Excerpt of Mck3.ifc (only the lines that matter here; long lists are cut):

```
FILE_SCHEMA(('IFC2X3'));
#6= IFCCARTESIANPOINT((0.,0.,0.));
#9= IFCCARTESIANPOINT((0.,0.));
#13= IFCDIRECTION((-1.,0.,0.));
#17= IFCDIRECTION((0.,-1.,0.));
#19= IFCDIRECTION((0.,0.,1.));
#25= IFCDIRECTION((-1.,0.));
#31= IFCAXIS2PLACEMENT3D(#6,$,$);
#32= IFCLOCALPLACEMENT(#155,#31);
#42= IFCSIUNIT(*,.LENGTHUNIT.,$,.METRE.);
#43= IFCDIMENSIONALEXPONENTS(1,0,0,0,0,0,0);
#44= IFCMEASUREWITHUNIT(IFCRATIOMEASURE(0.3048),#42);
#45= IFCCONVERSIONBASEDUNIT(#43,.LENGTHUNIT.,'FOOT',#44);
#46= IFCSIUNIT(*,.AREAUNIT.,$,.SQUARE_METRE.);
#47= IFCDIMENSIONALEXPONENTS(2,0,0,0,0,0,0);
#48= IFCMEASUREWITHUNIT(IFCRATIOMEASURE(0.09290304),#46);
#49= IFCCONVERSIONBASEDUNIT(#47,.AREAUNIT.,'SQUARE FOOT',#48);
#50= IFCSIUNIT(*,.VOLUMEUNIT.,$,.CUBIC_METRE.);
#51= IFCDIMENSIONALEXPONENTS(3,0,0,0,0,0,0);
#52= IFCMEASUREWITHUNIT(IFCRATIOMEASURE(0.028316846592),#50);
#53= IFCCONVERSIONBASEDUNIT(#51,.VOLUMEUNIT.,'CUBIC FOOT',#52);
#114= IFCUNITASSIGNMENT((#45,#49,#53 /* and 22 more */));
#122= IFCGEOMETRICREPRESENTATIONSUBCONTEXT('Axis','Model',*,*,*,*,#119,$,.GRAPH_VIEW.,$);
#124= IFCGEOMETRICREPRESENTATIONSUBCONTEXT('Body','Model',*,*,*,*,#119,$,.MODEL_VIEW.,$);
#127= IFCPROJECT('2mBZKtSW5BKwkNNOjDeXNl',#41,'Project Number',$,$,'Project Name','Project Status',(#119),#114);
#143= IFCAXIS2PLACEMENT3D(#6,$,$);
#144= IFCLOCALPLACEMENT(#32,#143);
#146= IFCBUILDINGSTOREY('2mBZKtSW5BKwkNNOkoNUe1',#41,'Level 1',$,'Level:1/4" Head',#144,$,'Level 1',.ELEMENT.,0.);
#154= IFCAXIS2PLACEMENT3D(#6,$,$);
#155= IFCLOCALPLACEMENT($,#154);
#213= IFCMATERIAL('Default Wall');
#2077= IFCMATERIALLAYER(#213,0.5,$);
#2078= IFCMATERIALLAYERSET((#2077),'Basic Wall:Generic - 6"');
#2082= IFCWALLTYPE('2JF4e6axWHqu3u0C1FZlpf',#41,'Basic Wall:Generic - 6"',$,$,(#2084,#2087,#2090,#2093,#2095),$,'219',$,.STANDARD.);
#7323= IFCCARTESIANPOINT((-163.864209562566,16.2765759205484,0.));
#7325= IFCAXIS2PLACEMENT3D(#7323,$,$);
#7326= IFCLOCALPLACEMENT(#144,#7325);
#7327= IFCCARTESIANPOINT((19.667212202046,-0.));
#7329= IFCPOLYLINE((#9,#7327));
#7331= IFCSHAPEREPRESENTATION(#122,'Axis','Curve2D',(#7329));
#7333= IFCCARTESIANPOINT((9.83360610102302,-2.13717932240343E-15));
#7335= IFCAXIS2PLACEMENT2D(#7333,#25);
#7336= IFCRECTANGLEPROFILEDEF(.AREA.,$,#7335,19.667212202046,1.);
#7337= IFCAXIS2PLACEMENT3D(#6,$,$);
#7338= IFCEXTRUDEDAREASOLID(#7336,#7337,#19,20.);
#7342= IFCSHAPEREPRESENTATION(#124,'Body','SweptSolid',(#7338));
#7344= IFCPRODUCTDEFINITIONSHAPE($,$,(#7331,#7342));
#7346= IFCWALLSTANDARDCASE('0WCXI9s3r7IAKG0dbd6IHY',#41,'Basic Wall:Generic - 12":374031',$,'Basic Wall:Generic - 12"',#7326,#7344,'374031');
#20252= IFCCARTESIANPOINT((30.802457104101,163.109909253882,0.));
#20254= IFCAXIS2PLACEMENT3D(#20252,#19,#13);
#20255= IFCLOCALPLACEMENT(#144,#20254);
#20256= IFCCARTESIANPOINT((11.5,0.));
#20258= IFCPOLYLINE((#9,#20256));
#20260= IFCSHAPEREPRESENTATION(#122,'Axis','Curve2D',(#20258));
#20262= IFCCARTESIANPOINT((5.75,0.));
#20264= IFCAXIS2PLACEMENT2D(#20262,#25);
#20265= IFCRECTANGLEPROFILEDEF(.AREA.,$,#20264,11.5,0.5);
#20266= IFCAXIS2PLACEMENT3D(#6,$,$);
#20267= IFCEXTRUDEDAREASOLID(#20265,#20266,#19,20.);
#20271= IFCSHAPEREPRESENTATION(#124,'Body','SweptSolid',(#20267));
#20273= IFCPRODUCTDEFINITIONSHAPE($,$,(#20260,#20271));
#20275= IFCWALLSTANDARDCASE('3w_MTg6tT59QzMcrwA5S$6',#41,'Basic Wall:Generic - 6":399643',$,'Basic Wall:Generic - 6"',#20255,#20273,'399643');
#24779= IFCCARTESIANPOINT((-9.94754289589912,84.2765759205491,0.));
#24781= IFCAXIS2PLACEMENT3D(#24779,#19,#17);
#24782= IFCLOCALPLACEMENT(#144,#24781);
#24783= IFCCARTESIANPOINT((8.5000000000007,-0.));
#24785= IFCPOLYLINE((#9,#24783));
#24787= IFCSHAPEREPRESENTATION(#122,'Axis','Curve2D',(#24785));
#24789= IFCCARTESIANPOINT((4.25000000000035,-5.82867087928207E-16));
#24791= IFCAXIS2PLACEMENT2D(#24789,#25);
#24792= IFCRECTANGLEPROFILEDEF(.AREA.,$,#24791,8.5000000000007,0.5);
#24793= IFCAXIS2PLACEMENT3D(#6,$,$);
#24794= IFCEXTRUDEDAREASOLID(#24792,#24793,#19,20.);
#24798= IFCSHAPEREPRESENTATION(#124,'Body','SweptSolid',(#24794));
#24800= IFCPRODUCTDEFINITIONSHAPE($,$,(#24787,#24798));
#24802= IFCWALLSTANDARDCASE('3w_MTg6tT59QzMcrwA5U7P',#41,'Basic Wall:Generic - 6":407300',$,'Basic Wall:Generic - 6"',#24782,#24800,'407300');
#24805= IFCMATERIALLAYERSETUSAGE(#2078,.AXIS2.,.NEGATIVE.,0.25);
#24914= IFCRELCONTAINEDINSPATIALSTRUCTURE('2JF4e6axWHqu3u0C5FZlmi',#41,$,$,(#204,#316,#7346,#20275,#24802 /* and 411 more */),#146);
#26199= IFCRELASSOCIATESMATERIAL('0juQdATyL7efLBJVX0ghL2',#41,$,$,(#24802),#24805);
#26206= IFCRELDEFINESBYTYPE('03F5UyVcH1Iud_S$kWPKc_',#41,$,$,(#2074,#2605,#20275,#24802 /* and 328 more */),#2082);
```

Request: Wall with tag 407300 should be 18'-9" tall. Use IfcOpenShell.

```python
import ifcopenshell
import ifcopenshell.geom
import ifcopenshell.util.representation
import ifcopenshell.util.shape
import ifcopenshell.util.unit

model = ifcopenshell.open("Mck3.ifc")
unit_scale = ifcopenshell.util.unit.calculate_unit_scale(model)
settings = ifcopenshell.geom.settings()


def volume(element):
    """Net volume in cubic metres, openings subtracted."""
    shape = ifcopenshell.geom.create_shape(settings, element)
    return ifcopenshell.util.shape.get_volume(shape.geometry)


wall = model.by_id(24802)
before = volume(wall)

body = ifcopenshell.util.representation.get_representation(wall, "Model", "Body")
solid = body.Items[0]
old_height = solid.Depth
solid.Depth = 225 * 0.0254 / unit_scale
after = volume(wall)

print(f"height {old_height:g} -> {solid.Depth:g}, volume {before:.3f} -> {after:.3f} m3")

model.write("Mck3_updated.ifc")
```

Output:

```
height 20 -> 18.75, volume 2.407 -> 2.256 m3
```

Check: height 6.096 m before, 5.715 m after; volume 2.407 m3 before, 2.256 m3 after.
